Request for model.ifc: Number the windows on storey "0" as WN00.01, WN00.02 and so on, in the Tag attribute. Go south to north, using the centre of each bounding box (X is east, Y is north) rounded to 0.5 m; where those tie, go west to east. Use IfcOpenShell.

First a look at what the model holds.

```python
import ifcopenshell
import ifcopenshell.util.element
import ifcopenshell.util.placement

model = ifcopenshell.open("model.ifc")
print(model.schema)
storey = next(s for s in model.by_type("IfcBuildingStorey") if s.Name == "0")
windows = [e for e in ifcopenshell.util.element.get_decomposition(storey) if e.is_a("IfcWindow")]
for e in sorted(windows, key=lambda e: e.id()):
    origin = ifcopenshell.util.placement.get_local_placement(e.ObjectPlacement)[:3, 3]
    print(e.id(), e.Tag, e.Name, origin.round(2) + 0.0, sep=" | ")
```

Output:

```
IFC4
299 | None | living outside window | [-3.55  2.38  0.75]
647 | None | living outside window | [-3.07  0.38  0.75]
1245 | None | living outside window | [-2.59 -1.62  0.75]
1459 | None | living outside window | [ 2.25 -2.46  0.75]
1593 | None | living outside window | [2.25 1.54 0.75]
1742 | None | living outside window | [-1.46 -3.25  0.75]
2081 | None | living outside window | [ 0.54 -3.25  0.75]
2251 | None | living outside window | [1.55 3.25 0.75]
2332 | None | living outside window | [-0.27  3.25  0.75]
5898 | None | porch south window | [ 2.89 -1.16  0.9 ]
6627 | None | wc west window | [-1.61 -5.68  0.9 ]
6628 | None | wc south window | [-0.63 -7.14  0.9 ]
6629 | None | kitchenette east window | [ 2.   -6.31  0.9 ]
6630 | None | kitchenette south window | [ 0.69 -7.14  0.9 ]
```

```python
import ifcopenshell
import ifcopenshell.geom
import ifcopenshell.util.element
import ifcopenshell.util.shape

model = ifcopenshell.open("model.ifc")
settings = ifcopenshell.geom.settings()
settings.set("use-world-coords", True)


def centre(element):
    shape = ifcopenshell.geom.create_shape(settings, element)
    return ifcopenshell.util.shape.get_bbox_centroid(shape.geometry)


storey = next(s for s in model.by_type("IfcBuildingStorey") if s.Name == "0")
windows = [e for e in ifcopenshell.util.element.get_decomposition(storey) if e.is_a("IfcWindow")]

# Insertion points can sit at a corner or the storey origin, so sort by the geometry (in metres).
centres = {e: centre(e) for e in windows}
windows.sort(key=lambda e: (round(centres[e][1] / 0.5), centres[e][0]))

for i, e in enumerate(windows, start=1):
    number = f"WN00.{i:02d}"
    e.Tag = number
    print(e.id(), number)

model.write("model_v2.ifc")
```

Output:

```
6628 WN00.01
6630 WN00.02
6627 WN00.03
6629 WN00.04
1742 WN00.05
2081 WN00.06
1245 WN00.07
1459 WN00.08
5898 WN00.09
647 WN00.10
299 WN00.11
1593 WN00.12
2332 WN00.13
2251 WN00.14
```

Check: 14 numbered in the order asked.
